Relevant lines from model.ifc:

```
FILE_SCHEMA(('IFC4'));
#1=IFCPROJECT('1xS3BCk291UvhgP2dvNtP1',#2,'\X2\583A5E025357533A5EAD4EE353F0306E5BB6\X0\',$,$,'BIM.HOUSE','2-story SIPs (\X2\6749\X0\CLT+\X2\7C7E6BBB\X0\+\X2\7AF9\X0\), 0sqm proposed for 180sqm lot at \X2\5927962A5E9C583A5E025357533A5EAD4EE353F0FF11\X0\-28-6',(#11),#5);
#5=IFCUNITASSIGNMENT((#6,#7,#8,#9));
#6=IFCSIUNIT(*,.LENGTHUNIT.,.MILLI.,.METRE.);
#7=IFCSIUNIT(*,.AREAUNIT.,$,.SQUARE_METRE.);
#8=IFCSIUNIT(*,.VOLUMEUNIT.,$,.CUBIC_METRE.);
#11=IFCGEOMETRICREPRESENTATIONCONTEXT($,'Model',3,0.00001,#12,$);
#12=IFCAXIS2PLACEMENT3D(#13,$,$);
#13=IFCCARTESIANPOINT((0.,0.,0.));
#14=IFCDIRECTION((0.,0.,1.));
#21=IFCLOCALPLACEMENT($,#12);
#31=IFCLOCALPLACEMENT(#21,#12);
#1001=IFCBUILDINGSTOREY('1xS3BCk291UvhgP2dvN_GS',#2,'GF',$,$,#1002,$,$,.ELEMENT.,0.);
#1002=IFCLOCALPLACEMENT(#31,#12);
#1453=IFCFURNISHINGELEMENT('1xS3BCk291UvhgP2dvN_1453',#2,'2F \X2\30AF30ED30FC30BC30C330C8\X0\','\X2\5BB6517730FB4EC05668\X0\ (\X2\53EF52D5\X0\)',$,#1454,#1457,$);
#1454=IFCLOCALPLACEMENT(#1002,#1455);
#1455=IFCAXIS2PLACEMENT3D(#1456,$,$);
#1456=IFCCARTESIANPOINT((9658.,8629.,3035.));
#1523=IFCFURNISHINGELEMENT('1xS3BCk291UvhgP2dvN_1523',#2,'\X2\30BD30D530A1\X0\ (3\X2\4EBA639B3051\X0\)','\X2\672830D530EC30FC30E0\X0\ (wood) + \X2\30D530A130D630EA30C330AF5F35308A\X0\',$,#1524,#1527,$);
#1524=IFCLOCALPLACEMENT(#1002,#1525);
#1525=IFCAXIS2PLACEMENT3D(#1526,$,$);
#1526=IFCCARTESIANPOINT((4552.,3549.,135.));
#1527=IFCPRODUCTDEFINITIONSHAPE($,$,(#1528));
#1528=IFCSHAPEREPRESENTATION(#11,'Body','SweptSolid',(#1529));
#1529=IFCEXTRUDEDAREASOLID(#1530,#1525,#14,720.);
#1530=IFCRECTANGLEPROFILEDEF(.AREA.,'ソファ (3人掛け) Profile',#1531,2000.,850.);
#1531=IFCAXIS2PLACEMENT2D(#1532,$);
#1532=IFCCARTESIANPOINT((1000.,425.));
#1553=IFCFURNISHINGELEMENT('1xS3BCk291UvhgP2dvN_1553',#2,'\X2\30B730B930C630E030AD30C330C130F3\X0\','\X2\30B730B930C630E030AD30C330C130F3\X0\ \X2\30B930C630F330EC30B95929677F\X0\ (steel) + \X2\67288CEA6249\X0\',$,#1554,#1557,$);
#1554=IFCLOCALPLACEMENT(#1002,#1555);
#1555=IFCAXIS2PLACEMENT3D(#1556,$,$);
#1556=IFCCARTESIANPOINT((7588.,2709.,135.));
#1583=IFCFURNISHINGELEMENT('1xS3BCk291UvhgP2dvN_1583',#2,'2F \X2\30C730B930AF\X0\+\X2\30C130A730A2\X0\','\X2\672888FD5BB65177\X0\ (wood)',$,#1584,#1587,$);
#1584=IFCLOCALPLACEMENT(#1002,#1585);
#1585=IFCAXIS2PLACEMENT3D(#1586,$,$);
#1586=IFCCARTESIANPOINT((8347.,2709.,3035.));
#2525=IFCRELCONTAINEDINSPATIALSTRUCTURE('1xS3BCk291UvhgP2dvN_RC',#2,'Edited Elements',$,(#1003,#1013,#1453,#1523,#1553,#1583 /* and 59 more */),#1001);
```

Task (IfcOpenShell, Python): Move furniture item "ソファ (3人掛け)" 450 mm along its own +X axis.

```python
import ifcopenshell
import ifcopenshell.api.geometry
import ifcopenshell.util.placement

model = ifcopenshell.open("model.ifc")

item = model.by_guid("1xS3BCk291UvhgP2dvN_1523")
matrix = ifcopenshell.util.placement.get_local_placement(item.ObjectPlacement)
matrix[:3, 3] += matrix[:3, 0] * 450.0
ifcopenshell.api.geometry.edit_object_placement(model, product=item, matrix=matrix, is_si=False)

print(ifcopenshell.util.placement.get_local_placement(item.ObjectPlacement).round(3) + 0.0)

model.write("model_v2.ifc")
```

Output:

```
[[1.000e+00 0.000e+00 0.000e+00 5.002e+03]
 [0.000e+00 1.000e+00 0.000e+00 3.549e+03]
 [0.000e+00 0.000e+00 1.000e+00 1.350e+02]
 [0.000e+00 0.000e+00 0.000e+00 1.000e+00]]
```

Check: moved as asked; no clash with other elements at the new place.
